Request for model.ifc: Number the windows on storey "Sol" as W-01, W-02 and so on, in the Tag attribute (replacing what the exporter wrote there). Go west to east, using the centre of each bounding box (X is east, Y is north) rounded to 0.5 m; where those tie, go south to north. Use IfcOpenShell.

First a look at what the model holds.

```python
import ifcopenshell
import ifcopenshell.util.element
import ifcopenshell.util.placement

model = ifcopenshell.open("model.ifc")
print(model.schema)
storey = next(s for s in model.by_type("IfcBuildingStorey") if s.Name == "Sol")
windows = [e for e in ifcopenshell.util.element.get_decomposition(storey) if e.is_a("IfcWindow")]
for e in sorted(windows, key=lambda e: e.id()):
    origin = ifcopenshell.util.placement.get_local_placement(e.ObjectPlacement)[:3, 3]
    print(e.id(), e.Tag, e.Name, origin.round(2) + 0.0, sep=" | ")
```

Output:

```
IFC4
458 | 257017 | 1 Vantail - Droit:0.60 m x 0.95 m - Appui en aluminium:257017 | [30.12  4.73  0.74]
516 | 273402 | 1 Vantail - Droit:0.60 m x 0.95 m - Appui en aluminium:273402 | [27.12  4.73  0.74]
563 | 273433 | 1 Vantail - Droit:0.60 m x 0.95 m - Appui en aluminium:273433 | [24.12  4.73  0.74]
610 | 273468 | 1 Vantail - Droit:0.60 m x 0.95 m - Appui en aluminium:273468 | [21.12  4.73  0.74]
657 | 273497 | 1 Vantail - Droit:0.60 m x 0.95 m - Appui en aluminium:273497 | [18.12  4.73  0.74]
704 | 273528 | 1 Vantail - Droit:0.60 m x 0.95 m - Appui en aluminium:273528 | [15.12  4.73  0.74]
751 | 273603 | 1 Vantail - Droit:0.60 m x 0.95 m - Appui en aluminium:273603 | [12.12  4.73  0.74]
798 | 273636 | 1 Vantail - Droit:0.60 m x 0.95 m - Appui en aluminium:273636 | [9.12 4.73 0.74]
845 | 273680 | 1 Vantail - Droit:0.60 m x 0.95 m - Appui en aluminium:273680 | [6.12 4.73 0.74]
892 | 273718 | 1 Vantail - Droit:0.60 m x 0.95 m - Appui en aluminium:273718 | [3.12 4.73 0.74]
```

```python
import ifcopenshell
import ifcopenshell.geom
import ifcopenshell.util.element
import ifcopenshell.util.shape

model = ifcopenshell.open("model.ifc")
settings = ifcopenshell.geom.settings()
settings.set("use-world-coords", True)


def centre(element):
    shape = ifcopenshell.geom.create_shape(settings, element)
    return ifcopenshell.util.shape.get_bbox_centroid(shape.geometry)


storey = next(s for s in model.by_type("IfcBuildingStorey") if s.Name == "Sol")
windows = [e for e in ifcopenshell.util.element.get_decomposition(storey) if e.is_a("IfcWindow")]

# Insertion points can sit at a corner or the storey origin, so sort by the geometry (in metres).
centres = {e: centre(e) for e in windows}
windows.sort(key=lambda e: (round(centres[e][0] / 0.5), centres[e][1]))

for i, e in enumerate(windows, start=1):
    number = f"W-{i:02d}"
    e.Tag = number
    print(e.id(), number)

model.write("model-out.ifc")
```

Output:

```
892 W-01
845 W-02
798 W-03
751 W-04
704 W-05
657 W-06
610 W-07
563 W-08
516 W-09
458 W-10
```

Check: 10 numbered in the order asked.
